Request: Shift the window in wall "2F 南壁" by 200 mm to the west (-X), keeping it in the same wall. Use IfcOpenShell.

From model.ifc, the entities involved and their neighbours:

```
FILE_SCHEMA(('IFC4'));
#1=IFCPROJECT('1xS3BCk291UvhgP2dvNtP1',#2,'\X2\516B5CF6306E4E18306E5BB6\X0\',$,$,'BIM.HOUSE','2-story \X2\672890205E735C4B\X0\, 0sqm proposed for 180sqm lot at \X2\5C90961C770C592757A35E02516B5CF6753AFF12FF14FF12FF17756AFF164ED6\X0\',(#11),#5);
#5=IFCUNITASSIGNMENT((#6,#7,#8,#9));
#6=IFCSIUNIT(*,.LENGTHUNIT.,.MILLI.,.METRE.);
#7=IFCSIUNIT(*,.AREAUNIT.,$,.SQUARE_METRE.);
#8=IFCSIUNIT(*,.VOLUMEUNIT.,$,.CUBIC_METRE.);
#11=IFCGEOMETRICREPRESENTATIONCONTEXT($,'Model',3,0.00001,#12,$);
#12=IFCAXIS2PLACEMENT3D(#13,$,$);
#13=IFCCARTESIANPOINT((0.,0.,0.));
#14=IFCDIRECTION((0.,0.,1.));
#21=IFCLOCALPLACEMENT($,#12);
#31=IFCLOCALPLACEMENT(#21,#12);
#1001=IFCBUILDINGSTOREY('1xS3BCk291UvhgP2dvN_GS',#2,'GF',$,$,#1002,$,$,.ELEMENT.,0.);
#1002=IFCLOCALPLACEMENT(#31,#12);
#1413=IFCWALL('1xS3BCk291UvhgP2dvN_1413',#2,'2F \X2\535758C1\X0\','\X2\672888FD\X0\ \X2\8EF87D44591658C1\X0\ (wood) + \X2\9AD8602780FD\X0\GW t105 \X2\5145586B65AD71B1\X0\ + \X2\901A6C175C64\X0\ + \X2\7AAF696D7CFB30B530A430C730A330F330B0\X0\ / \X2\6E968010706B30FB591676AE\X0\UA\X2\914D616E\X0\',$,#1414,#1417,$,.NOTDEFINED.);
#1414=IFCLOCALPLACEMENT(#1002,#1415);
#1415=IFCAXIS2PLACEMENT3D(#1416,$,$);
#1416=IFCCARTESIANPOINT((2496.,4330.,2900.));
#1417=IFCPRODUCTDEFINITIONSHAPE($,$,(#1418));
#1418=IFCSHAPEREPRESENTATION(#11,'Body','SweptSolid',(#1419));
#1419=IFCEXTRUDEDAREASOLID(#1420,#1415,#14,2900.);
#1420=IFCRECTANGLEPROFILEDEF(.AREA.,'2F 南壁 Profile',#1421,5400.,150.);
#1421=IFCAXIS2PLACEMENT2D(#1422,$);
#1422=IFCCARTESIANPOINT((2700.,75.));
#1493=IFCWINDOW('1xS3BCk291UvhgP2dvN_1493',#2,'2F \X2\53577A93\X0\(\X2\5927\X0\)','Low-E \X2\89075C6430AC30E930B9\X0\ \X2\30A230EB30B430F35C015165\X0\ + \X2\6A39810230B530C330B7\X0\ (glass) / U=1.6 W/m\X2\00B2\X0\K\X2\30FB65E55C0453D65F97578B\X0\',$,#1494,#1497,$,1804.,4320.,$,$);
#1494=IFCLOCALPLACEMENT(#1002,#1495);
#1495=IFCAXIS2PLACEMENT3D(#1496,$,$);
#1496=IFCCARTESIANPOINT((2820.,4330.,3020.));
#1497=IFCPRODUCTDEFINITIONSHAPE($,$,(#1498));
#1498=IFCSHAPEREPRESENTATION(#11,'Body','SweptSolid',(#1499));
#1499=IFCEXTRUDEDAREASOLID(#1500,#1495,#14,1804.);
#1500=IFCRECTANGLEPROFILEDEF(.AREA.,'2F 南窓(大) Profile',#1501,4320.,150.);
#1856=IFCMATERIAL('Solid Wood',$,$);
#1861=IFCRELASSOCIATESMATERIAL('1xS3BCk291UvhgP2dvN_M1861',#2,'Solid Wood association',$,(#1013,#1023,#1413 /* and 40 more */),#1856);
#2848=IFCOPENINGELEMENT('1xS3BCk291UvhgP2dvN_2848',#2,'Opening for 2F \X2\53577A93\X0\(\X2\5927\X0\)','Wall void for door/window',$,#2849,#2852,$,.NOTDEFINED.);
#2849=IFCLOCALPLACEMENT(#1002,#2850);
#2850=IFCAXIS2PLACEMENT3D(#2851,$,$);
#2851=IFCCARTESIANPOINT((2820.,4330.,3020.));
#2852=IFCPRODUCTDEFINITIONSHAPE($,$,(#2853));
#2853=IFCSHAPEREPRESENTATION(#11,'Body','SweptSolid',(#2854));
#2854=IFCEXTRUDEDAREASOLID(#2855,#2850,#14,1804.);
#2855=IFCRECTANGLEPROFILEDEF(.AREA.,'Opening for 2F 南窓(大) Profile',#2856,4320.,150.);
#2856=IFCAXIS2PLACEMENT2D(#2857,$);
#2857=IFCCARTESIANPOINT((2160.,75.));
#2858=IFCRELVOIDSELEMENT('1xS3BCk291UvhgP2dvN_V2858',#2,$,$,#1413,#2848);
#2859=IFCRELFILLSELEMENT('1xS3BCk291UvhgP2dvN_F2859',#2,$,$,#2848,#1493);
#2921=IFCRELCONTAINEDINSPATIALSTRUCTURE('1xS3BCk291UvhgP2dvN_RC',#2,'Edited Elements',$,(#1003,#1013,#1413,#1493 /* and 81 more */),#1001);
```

```python
import ifcopenshell
import ifcopenshell.api.geometry
import ifcopenshell.util.placement

model = ifcopenshell.open("model.ifc")

window = model.by_guid("1xS3BCk291UvhgP2dvN_1493")
opening = window.FillsVoids[0].RelatingOpeningElement
wall = opening.VoidsElements[0].RelatingBuildingElement

wall_matrix = ifcopenshell.util.placement.get_local_placement(wall.ObjectPlacement)
shift = wall_matrix[:3, 0] * -200.0
before = ifcopenshell.util.placement.get_local_placement(window.ObjectPlacement)[:3, 3].copy()

# The window is not placed relative to its opening, so move both.
for product in (opening, window):
    matrix = ifcopenshell.util.placement.get_local_placement(product.ObjectPlacement)
    matrix[:3, 3] += shift
    ifcopenshell.api.geometry.edit_object_placement(model, product=product, matrix=matrix, is_si=False)

after = ifcopenshell.util.placement.get_local_placement(window.ObjectPlacement)[:3, 3]
print("window moved by", (after - before).round(3) + 0.0)

model.write("model_edited.ifc")
```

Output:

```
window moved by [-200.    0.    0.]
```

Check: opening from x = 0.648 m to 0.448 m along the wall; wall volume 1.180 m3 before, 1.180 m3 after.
